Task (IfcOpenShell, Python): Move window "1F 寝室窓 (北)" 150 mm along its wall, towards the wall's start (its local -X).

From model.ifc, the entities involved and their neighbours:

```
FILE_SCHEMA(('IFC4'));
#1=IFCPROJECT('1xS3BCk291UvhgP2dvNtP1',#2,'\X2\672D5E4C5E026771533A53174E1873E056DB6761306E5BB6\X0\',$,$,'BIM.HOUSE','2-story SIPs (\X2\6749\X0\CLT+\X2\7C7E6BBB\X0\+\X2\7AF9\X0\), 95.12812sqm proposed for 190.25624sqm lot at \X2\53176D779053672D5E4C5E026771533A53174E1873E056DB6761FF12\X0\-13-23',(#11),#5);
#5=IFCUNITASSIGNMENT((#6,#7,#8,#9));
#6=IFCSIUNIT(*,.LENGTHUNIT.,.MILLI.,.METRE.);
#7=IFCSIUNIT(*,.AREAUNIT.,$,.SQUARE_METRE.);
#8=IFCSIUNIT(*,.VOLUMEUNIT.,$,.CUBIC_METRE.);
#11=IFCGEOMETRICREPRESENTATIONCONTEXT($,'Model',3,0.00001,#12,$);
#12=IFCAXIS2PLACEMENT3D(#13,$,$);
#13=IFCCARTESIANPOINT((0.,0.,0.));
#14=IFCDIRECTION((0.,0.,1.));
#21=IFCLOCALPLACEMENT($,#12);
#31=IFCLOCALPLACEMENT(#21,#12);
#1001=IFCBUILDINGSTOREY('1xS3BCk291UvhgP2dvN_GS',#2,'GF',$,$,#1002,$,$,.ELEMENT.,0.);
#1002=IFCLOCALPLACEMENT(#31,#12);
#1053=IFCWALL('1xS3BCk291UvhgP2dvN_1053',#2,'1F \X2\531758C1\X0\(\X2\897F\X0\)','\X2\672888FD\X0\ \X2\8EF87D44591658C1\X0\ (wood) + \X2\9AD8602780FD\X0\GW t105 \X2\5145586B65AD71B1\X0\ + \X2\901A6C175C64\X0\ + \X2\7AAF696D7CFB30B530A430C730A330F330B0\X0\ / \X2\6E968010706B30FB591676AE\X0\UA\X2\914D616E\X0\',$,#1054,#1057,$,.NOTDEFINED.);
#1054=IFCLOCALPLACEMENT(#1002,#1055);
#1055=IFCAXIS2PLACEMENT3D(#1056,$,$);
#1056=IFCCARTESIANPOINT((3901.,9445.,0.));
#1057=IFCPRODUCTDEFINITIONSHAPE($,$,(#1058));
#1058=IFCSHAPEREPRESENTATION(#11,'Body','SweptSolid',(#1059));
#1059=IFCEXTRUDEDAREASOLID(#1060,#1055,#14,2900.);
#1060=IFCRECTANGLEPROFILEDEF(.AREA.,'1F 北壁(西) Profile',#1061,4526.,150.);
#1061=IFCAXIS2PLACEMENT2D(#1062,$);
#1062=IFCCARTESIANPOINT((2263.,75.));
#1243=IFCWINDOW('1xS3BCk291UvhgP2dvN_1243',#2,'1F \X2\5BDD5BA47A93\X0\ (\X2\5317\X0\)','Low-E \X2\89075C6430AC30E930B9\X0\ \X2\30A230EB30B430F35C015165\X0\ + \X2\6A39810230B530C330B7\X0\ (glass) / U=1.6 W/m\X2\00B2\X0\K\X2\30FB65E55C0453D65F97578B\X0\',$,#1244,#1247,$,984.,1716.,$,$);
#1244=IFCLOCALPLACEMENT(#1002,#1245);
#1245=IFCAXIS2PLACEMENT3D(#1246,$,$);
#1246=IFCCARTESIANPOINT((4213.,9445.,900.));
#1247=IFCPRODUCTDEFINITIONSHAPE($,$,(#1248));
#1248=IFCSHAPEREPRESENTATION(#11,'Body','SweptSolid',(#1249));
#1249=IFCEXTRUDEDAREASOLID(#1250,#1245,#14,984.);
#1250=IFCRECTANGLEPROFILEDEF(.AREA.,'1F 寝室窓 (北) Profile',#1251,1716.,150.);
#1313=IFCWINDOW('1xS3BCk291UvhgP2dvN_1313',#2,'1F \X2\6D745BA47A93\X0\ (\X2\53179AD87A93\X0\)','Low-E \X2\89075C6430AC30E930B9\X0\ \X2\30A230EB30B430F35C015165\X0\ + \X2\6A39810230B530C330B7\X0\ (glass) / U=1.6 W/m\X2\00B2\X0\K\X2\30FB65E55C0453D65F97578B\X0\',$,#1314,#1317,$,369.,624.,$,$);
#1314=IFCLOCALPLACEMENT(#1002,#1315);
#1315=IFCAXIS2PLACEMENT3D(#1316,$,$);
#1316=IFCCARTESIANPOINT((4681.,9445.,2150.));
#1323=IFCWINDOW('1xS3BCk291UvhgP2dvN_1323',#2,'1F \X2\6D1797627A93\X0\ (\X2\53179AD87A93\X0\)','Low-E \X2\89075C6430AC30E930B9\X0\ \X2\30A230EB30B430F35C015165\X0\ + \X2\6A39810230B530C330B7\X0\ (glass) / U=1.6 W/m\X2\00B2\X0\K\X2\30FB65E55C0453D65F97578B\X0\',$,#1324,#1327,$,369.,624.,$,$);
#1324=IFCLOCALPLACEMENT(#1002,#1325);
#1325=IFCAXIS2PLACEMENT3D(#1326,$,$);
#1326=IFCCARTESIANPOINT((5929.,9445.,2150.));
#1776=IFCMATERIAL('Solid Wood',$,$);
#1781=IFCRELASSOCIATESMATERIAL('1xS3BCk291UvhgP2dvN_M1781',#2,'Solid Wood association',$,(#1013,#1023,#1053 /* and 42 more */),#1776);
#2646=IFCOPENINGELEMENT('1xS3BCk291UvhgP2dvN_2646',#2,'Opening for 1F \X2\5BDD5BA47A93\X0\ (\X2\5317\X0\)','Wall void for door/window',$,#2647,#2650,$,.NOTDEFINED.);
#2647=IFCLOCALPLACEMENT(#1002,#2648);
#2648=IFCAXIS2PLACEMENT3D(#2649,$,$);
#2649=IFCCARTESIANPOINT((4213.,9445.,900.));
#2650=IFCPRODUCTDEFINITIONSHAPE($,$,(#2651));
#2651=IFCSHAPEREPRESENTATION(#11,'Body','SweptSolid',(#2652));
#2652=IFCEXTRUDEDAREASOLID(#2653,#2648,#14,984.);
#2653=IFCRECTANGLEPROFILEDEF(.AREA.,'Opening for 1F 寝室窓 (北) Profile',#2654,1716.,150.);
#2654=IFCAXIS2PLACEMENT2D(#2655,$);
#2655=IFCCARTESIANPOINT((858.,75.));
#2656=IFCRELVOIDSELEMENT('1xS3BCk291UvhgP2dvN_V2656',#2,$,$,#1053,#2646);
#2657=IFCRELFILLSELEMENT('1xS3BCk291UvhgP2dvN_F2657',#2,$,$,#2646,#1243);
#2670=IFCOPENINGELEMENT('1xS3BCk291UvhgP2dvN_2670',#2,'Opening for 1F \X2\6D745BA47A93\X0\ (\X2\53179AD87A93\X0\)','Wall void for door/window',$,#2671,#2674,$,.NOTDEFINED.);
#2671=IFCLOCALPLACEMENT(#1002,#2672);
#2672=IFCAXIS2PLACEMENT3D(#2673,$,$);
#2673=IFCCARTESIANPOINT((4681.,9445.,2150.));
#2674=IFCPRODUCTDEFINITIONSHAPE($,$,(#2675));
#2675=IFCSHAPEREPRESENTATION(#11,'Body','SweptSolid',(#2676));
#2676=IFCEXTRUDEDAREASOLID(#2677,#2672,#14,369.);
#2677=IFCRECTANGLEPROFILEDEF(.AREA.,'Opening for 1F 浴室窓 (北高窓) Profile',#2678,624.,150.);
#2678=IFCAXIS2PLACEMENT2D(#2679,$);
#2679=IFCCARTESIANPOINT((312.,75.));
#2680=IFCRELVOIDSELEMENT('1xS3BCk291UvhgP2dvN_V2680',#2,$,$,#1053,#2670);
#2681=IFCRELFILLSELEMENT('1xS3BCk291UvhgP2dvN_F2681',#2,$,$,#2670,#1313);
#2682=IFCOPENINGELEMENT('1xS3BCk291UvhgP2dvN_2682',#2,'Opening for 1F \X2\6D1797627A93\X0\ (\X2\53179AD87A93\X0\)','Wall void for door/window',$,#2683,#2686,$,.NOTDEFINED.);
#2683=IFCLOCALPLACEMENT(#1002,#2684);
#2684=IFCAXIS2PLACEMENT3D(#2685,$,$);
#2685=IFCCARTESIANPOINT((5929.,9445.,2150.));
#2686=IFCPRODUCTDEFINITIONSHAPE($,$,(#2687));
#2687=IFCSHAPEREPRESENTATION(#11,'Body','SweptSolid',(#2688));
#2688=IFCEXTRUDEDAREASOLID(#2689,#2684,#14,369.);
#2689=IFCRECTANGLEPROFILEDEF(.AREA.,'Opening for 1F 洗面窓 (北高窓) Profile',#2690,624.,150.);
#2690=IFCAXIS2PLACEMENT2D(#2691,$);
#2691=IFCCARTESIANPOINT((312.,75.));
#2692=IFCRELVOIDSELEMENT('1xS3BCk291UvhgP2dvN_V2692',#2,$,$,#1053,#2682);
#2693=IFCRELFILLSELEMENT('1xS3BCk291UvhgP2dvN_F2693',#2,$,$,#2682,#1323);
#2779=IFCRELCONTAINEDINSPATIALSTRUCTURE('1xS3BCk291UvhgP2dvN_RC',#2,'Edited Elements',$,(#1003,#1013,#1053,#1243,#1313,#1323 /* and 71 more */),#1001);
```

```python
import ifcopenshell
import ifcopenshell.api.geometry
import ifcopenshell.util.placement
import ifcopenshell.util.unit

model = ifcopenshell.open("model.ifc")
unit_scale = ifcopenshell.util.unit.calculate_unit_scale(model)

window = model.by_id(1243)
opening = window.FillsVoids[0].RelatingOpeningElement
wall = opening.VoidsElements[0].RelatingBuildingElement

wall_matrix = ifcopenshell.util.placement.get_local_placement(wall.ObjectPlacement)
shift = wall_matrix[:3, 0] * -0.15 / unit_scale
before = ifcopenshell.util.placement.get_local_placement(window.ObjectPlacement)[:3, 3].copy()

# The window is not placed relative to its opening, so move both.
for product in (opening, window):
    matrix = ifcopenshell.util.placement.get_local_placement(product.ObjectPlacement)
    matrix[:3, 3] += shift
    ifcopenshell.api.geometry.edit_object_placement(model, product=product, matrix=matrix, is_si=False)

after = ifcopenshell.util.placement.get_local_placement(window.ObjectPlacement)[:3, 3]
print("window moved by", (after - before).round(3) + 0.0)

model.write("model_v2.ifc")
```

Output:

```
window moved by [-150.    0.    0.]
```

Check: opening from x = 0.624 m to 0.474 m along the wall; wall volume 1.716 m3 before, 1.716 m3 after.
